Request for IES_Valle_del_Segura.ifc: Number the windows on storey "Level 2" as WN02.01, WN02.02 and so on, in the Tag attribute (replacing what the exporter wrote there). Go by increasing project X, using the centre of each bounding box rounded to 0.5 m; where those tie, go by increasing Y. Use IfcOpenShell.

First a look at what the model holds.

```python
import ifcopenshell
import ifcopenshell.util.element
import ifcopenshell.util.placement

model = ifcopenshell.open("IES_Valle_del_Segura.ifc")
print(model.schema)
storey = next(s for s in model.by_type("IfcBuildingStorey") if s.Name == "Level 2")
windows = [e for e in ifcopenshell.util.element.get_decomposition(storey) if e.is_a("IfcWindow")]
for e in sorted(windows, key=lambda e: e.id()):
    origin = ifcopenshell.util.placement.get_local_placement(e.ObjectPlacement)[:3, 3]
    print(e.id(), e.Tag, e.Name, origin.round(2) + 0.0, sep=" | ")
```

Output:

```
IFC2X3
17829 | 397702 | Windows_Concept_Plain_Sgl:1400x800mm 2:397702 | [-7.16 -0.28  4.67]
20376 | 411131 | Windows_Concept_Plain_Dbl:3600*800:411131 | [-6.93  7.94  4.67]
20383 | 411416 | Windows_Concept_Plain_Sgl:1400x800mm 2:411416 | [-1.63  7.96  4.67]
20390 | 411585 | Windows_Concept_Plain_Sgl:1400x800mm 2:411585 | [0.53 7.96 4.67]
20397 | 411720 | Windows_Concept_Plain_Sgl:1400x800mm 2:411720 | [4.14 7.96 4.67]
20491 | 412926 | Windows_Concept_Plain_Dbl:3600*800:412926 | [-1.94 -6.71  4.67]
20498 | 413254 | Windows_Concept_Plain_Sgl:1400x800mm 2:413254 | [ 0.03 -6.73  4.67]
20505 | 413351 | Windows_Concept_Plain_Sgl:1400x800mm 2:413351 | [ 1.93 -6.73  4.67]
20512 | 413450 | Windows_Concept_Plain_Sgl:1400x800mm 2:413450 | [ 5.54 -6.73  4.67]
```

```python
import ifcopenshell
import ifcopenshell.geom
import ifcopenshell.util.element
import ifcopenshell.util.shape

model = ifcopenshell.open("IES_Valle_del_Segura.ifc")
settings = ifcopenshell.geom.settings()
settings.set("use-world-coords", True)


def centre(element):
    shape = ifcopenshell.geom.create_shape(settings, element)
    return ifcopenshell.util.shape.get_bbox_centroid(shape.geometry)


storey = next(s for s in model.by_type("IfcBuildingStorey") if s.Name == "Level 2")
windows = [e for e in ifcopenshell.util.element.get_decomposition(storey) if e.is_a("IfcWindow")]

# Insertion points can sit at a corner or the storey origin, so sort by the geometry (in metres).
centres = {e: centre(e) for e in windows}
windows.sort(key=lambda e: (round(centres[e][0] / 0.5), centres[e][1]))

for i, e in enumerate(windows, start=1):
    number = f"WN02.{i:02d}"
    e.Tag = number
    print(e.id(), number)

model.write("IES_Valle_del_Segura_updated.ifc")
```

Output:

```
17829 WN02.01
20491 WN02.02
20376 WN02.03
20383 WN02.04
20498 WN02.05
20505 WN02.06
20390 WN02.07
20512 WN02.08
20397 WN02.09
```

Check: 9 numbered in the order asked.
